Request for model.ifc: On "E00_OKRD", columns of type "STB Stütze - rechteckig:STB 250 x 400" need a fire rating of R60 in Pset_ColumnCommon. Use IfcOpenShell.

First a look at what the model holds.

```python
import ifcopenshell
import ifcopenshell.util.element

model = ifcopenshell.open("model.ifc")
print(model.schema)
storey = next(s for s in model.by_type("IfcBuildingStorey") if s.Name == "E00_OKRD")
columns = [e for e in ifcopenshell.util.element.get_decomposition(storey) if e.is_a("IfcColumn")]
seen = {}
for e in columns:
    element_type = ifcopenshell.util.element.get_type(e)
    key = (element_type.Name if element_type != e and element_type else None, ifcopenshell.util.element.get_pset(e, "Pset_ColumnCommon", "FireRating"))
    seen[key] = seen.get(key, 0) + 1
for (name, value), count in sorted(seen.items(), key=str):
    print(count, "x", name, "|", value)
```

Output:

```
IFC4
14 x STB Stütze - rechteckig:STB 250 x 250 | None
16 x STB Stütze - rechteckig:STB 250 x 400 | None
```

```python
import ifcopenshell
import ifcopenshell.api.pset
import ifcopenshell.util.element

model = ifcopenshell.open("model.ifc")

storey = next(s for s in model.by_type("IfcBuildingStorey") if s.Name == "E00_OKRD")
columns = [e for e in ifcopenshell.util.element.get_decomposition(storey) if e.is_a("IfcColumn")]

count = 0
for e in columns:
    element_type = ifcopenshell.util.element.get_type(e)
    if element_type in (None, e) or element_type.Name != "STB Stütze - rechteckig:STB 250 x 400":
        continue
    # add_pset returns the element's existing set when there is one.
    pset = ifcopenshell.api.pset.add_pset(model, product=e, name="Pset_ColumnCommon")
    ifcopenshell.api.pset.edit_pset(model, pset=pset, properties={"FireRating": "R60"})
    count += 1

print(count, "columns updated")

model.write("model-out.ifc")
```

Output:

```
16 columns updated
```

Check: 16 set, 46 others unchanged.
